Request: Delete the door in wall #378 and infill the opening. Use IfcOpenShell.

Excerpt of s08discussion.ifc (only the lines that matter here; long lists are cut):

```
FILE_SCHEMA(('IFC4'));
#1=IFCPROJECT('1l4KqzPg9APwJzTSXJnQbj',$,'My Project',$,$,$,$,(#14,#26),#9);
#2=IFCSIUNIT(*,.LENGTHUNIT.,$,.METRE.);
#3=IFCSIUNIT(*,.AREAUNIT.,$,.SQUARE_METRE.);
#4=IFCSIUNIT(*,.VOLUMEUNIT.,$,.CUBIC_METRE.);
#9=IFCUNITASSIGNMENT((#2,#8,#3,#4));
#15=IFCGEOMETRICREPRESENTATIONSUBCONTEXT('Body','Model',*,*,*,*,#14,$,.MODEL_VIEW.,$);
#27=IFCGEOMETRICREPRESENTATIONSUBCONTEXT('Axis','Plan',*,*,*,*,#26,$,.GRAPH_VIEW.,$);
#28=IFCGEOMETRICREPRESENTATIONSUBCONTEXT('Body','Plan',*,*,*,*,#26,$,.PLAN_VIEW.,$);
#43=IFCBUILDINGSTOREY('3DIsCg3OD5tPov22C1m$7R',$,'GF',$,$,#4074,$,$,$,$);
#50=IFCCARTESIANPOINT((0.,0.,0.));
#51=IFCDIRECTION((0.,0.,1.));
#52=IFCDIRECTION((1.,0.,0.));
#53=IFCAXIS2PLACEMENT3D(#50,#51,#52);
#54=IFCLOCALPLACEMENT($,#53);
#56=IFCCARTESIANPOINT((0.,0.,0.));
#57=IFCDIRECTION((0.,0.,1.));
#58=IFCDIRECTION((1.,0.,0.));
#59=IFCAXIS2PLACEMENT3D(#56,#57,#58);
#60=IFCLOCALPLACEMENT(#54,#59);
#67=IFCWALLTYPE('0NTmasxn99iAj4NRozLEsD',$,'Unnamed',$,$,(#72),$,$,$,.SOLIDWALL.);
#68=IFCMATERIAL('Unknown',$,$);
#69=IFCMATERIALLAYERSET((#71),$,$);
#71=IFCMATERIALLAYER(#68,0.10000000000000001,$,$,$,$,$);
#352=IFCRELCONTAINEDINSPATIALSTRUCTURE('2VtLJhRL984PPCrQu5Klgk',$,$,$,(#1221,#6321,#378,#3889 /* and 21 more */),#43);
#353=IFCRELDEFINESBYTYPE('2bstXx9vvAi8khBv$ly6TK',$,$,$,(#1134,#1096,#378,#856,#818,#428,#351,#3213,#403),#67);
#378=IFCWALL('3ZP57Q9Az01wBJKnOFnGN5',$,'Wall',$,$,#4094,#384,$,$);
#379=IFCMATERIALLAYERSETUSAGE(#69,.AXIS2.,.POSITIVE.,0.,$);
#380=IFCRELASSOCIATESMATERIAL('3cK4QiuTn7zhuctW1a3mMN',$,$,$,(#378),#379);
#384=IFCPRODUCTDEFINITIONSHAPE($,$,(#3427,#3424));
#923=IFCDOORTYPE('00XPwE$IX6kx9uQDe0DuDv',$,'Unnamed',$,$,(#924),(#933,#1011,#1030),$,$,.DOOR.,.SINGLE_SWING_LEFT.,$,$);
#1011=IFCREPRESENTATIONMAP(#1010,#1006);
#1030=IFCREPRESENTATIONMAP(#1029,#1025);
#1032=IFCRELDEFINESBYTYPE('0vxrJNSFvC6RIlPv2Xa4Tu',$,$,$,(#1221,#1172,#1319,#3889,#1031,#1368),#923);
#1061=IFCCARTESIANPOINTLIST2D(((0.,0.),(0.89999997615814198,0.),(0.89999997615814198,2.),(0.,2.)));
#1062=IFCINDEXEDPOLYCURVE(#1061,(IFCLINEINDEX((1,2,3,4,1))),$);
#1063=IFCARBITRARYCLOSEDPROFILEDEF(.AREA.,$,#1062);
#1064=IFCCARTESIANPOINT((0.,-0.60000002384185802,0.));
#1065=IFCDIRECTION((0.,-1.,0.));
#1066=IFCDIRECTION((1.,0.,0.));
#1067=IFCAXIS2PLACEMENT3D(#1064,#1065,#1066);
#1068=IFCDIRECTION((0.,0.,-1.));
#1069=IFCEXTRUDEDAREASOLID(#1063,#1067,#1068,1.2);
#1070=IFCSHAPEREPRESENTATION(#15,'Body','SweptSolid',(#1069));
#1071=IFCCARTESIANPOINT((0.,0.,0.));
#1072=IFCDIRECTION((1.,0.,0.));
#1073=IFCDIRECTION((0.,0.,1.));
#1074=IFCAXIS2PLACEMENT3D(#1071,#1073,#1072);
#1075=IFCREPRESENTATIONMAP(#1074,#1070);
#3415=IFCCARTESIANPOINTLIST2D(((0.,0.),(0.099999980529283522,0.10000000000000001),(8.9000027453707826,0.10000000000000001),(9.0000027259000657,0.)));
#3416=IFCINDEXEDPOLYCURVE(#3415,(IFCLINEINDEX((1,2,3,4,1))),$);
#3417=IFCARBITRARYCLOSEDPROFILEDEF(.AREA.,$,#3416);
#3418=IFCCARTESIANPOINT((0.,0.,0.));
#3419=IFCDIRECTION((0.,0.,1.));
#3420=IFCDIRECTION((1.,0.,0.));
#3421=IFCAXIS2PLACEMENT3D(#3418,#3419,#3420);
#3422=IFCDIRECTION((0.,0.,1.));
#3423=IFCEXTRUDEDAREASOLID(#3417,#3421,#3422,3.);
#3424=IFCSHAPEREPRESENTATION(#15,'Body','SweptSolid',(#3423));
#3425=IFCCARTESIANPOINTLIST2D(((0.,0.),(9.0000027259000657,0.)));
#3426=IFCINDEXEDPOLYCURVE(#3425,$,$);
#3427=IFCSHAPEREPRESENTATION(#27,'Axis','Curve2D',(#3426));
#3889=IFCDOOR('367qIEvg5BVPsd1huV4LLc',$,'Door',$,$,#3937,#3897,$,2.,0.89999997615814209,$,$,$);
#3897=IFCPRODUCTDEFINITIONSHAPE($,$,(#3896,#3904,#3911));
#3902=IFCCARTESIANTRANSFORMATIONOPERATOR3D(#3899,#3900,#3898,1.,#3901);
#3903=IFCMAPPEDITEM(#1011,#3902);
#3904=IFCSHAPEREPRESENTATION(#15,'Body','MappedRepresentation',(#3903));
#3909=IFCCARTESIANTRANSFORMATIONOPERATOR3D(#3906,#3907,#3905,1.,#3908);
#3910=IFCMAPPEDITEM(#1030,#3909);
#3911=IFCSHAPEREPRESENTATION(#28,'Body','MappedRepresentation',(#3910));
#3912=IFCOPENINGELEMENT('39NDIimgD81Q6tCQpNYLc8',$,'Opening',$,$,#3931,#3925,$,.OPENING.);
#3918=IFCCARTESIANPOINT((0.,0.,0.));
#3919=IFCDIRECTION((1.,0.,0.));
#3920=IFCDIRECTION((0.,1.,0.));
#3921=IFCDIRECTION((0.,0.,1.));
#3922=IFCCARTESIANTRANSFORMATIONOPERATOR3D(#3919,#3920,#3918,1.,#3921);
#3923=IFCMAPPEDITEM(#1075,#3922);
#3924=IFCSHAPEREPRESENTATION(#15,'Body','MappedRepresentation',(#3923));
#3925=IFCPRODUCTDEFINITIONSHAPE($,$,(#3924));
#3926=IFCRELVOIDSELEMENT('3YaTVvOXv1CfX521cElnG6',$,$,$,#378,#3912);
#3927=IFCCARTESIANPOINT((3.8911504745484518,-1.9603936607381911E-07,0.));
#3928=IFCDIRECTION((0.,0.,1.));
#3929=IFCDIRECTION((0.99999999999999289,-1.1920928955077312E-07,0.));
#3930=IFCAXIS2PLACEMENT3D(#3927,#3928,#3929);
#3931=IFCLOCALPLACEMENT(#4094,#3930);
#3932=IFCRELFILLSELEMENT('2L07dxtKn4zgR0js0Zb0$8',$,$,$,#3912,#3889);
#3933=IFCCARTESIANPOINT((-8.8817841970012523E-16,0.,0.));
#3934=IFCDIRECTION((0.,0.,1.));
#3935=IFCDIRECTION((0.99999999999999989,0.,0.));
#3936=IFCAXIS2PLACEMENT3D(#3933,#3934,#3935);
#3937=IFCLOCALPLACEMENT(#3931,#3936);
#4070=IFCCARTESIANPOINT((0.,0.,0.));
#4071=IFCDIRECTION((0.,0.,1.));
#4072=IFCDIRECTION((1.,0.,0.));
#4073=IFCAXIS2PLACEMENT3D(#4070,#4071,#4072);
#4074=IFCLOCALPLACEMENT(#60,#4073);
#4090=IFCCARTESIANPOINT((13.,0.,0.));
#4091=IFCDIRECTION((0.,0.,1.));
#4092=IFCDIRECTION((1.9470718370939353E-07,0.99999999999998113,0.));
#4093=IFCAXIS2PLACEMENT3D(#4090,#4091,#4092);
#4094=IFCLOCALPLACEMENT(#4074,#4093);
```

```python
import ifcopenshell
import ifcopenshell.api.feature
import ifcopenshell.api.root
import ifcopenshell.geom
import ifcopenshell.util.shape

model = ifcopenshell.open("s08discussion.ifc")
settings = ifcopenshell.geom.settings()


def volume(element):
    """Net volume in cubic metres, openings subtracted."""
    shape = ifcopenshell.geom.create_shape(settings, element)
    return ifcopenshell.util.shape.get_volume(shape.geometry)


door = model.by_guid("367qIEvg5BVPsd1huV4LLc")
opening = door.FillsVoids[0].RelatingOpeningElement
wall = opening.VoidsElements[0].RelatingBuildingElement
before = volume(wall)

ifcopenshell.api.root.remove_product(model, product=door)
ifcopenshell.api.feature.remove_feature(model, feature=opening)

after = volume(wall)

print(f"wall volume {before:.3f} -> {after:.3f} m3")

model.write("s08discussion_updated.ifc")
```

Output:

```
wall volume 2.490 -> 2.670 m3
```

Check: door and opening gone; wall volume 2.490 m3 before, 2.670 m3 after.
